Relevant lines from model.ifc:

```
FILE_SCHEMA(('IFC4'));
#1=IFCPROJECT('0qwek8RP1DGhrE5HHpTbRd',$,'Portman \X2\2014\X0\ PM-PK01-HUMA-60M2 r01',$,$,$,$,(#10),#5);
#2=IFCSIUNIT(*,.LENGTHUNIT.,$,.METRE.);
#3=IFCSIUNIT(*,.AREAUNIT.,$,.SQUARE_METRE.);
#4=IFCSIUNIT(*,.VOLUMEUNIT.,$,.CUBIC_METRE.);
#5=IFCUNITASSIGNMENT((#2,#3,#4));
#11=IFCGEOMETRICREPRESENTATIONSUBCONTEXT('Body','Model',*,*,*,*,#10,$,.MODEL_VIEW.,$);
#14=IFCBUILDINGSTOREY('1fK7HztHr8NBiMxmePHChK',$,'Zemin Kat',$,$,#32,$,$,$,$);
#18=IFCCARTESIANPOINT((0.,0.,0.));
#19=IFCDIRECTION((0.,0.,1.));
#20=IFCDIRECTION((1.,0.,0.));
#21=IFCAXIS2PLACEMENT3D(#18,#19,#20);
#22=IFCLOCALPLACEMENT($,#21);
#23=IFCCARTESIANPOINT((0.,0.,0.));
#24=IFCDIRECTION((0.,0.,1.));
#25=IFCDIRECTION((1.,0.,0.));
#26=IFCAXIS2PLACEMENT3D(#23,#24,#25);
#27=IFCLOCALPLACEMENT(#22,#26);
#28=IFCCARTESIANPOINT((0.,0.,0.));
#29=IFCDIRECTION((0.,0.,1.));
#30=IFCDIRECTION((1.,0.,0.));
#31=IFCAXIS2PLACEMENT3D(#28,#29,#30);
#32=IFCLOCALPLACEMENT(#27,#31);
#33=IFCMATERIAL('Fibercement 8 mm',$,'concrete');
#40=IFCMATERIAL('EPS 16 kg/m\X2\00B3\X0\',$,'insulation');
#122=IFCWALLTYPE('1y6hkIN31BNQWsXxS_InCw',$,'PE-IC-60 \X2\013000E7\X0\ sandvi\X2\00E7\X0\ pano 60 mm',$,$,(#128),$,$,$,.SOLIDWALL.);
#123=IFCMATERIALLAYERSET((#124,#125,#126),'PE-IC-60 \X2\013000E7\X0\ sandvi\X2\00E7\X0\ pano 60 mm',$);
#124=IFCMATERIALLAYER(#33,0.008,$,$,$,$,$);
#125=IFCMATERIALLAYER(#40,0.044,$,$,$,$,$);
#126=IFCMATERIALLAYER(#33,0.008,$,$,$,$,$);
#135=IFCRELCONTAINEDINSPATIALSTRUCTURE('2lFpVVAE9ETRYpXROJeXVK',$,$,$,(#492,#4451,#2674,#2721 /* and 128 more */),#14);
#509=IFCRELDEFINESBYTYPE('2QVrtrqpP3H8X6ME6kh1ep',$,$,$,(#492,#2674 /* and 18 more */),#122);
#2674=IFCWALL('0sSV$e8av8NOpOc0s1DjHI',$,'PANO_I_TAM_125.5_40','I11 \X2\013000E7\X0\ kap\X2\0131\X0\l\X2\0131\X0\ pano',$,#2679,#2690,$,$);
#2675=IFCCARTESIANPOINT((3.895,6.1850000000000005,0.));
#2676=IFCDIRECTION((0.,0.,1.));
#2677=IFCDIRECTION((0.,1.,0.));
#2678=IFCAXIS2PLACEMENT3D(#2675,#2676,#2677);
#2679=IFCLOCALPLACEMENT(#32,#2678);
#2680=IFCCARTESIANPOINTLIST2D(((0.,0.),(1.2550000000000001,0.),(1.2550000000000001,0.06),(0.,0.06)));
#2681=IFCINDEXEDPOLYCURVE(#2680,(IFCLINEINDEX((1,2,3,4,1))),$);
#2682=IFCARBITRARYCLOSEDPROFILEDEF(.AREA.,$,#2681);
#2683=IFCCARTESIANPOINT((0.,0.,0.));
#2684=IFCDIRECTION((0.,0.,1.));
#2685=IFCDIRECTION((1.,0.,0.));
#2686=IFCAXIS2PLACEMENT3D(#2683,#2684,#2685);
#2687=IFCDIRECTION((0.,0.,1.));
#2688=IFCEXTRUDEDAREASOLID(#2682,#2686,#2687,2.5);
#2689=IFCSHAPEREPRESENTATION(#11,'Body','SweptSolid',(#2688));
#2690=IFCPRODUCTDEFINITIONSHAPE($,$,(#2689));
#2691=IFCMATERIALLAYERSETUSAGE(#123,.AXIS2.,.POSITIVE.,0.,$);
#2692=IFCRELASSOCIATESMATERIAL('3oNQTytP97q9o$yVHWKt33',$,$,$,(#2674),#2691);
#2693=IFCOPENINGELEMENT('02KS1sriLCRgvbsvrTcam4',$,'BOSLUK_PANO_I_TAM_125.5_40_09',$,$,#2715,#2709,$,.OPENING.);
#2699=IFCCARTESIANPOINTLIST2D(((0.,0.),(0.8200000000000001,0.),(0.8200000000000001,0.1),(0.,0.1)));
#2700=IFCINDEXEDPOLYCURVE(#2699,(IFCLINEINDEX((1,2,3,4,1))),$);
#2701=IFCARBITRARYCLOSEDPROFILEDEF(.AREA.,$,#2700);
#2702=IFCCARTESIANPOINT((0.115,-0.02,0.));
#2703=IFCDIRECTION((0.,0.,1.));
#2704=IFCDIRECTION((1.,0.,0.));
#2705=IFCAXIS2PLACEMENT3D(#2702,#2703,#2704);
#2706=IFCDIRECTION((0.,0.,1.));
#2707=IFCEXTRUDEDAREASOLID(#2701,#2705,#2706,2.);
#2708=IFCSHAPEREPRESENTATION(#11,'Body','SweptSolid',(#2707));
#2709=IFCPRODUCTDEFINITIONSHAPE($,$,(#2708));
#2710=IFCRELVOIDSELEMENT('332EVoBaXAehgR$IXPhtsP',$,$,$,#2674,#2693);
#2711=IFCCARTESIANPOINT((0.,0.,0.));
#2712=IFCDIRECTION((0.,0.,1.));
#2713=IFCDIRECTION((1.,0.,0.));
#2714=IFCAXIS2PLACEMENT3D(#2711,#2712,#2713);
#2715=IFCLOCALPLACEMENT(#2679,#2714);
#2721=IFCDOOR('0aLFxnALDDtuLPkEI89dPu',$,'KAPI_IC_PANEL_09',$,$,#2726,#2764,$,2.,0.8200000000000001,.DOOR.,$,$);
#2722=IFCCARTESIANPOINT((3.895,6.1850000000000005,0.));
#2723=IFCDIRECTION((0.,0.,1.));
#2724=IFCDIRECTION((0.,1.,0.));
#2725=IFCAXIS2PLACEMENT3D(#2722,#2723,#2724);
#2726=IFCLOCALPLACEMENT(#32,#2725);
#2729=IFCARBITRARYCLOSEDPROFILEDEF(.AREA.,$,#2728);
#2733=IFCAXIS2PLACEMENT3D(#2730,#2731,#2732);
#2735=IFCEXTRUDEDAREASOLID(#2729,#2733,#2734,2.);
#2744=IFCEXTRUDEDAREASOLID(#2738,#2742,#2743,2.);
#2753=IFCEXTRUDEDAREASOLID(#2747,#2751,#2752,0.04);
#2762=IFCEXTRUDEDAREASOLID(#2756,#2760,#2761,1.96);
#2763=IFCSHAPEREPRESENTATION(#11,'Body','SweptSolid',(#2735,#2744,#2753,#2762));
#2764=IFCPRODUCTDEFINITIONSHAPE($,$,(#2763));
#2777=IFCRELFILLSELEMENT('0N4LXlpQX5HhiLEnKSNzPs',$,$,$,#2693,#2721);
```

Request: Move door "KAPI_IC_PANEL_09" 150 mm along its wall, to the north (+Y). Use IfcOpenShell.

```python
import ifcopenshell
import ifcopenshell.api.geometry
import ifcopenshell.util.placement
import ifcopenshell.util.unit

model = ifcopenshell.open("model.ifc")
unit_scale = ifcopenshell.util.unit.calculate_unit_scale(model)

door = model.by_id(2721)
opening = door.FillsVoids[0].RelatingOpeningElement
wall = opening.VoidsElements[0].RelatingBuildingElement

wall_matrix = ifcopenshell.util.placement.get_local_placement(wall.ObjectPlacement)
shift = wall_matrix[:3, 0] * 0.15 / unit_scale
before = ifcopenshell.util.placement.get_local_placement(door.ObjectPlacement)[:3, 3].copy()

# The door is not placed relative to its opening, so move both.
for product in (opening, door):
    matrix = ifcopenshell.util.placement.get_local_placement(product.ObjectPlacement)
    matrix[:3, 3] += shift
    ifcopenshell.api.geometry.edit_object_placement(model, product=product, matrix=matrix, is_si=False)

after = ifcopenshell.util.placement.get_local_placement(door.ObjectPlacement)[:3, 3]
print("door moved by", (after - before).round(3) + 0.0)

model.write("model_rev.ifc")
```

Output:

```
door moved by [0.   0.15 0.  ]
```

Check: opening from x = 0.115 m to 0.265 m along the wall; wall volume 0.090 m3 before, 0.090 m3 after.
